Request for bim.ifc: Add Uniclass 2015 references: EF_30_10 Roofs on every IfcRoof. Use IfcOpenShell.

First a look at what the model holds.

```python
import ifcopenshell

model = ifcopenshell.open("bim.ifc")
print(model.schema)
print("classifications:", [c.Name for c in model.by_type("IfcClassification")])
for ifc_class in ("IfcDoor", "IfcRoof", "IfcStair", "IfcWall", "IfcWindow"):
    print(ifc_class, len(model.by_type(ifc_class)))
```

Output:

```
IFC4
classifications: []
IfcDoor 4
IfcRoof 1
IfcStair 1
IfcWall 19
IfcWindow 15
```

```python
import ifcopenshell
import ifcopenshell.api.classification

model = ifcopenshell.open("bim.ifc")

system = ifcopenshell.api.classification.add_classification(model, classification="Uniclass 2015")

codes = {
    "IfcRoof": ("EF_30_10", "Roofs"),
}
for ifc_class, (code, name) in codes.items():
    products = model.by_type(ifc_class)
    ifcopenshell.api.classification.add_reference(
        model, products=products, classification=system, identification=code, name=name
    )
    print(code, len(products))

model.write("bim_edited.ifc")
```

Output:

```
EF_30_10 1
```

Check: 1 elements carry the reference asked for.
